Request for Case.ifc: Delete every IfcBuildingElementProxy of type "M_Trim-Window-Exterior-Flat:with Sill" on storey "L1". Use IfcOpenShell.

First a look at what the model holds.

```python
import ifcopenshell
import ifcopenshell.util.element

model = ifcopenshell.open("Case.ifc")
print(model.schema)
storey = next(s for s in model.by_type("IfcBuildingStorey") if s.Name == "L1")
proxies = [e for e in ifcopenshell.util.element.get_decomposition(storey) if e.is_a("IfcBuildingElementProxy")]
seen = {}
for e in proxies:
    element_type = ifcopenshell.util.element.get_type(e)
    name = element_type.Name if element_type not in (None, e) else None
    seen[name] = seen.get(name, 0) + 1
for name, count in sorted(seen.items(), key=str):
    print(count, "x", name)
```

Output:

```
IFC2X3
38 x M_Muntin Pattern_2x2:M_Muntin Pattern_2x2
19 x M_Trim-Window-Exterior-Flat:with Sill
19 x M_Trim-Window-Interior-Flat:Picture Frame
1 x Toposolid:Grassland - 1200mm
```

```python
import ifcopenshell
import ifcopenshell.api.root
import ifcopenshell.util.element

model = ifcopenshell.open("Case.ifc")

storey = next(s for s in model.by_type("IfcBuildingStorey") if s.Name == "L1")
proxies = [e for e in ifcopenshell.util.element.get_decomposition(storey) if e.is_a("IfcBuildingElementProxy")]
targets = [e for e in proxies if (t := ifcopenshell.util.element.get_type(e)) not in (None, e) and t.Name == "M_Trim-Window-Exterior-Flat:with Sill"]

for e in targets:
    ifcopenshell.api.root.remove_product(model, product=e)
print(len(targets), "removed")

model.write("Case_v2.ifc")
```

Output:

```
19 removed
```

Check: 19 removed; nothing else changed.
